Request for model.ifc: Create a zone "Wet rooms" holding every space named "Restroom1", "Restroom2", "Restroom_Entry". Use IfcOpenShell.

First a look at what the model holds.

```python
import ifcopenshell

model = ifcopenshell.open("model.ifc")
print(model.schema)
seen = {}
for space in model.by_type("IfcSpace"):
    seen[space.LongName] = seen.get(space.LongName, 0) + 1
for name, count in sorted(seen.items(), key=str):
    print(count, "x", name)
print("zones:", [z.Name for z in model.by_type("IfcZone")][:20])
```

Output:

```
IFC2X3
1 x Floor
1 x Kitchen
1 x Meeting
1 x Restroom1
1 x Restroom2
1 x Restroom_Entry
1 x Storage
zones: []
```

```python
import ifcopenshell
import ifcopenshell.api.group
import ifcopenshell.api.root

model = ifcopenshell.open("model.ifc")

names = {"Restroom1", "Restroom2", "Restroom_Entry"}
spaces = [s for s in model.by_type("IfcSpace") if s.LongName in names]

zone = ifcopenshell.api.root.create_entity(model, ifc_class="IfcZone", name="Wet rooms")
ifcopenshell.api.group.assign_group(model, products=spaces, group=zone)
print(len(spaces), "spaces in", zone.Name)

model.write("model_rev.ifc")
```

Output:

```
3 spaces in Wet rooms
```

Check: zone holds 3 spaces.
